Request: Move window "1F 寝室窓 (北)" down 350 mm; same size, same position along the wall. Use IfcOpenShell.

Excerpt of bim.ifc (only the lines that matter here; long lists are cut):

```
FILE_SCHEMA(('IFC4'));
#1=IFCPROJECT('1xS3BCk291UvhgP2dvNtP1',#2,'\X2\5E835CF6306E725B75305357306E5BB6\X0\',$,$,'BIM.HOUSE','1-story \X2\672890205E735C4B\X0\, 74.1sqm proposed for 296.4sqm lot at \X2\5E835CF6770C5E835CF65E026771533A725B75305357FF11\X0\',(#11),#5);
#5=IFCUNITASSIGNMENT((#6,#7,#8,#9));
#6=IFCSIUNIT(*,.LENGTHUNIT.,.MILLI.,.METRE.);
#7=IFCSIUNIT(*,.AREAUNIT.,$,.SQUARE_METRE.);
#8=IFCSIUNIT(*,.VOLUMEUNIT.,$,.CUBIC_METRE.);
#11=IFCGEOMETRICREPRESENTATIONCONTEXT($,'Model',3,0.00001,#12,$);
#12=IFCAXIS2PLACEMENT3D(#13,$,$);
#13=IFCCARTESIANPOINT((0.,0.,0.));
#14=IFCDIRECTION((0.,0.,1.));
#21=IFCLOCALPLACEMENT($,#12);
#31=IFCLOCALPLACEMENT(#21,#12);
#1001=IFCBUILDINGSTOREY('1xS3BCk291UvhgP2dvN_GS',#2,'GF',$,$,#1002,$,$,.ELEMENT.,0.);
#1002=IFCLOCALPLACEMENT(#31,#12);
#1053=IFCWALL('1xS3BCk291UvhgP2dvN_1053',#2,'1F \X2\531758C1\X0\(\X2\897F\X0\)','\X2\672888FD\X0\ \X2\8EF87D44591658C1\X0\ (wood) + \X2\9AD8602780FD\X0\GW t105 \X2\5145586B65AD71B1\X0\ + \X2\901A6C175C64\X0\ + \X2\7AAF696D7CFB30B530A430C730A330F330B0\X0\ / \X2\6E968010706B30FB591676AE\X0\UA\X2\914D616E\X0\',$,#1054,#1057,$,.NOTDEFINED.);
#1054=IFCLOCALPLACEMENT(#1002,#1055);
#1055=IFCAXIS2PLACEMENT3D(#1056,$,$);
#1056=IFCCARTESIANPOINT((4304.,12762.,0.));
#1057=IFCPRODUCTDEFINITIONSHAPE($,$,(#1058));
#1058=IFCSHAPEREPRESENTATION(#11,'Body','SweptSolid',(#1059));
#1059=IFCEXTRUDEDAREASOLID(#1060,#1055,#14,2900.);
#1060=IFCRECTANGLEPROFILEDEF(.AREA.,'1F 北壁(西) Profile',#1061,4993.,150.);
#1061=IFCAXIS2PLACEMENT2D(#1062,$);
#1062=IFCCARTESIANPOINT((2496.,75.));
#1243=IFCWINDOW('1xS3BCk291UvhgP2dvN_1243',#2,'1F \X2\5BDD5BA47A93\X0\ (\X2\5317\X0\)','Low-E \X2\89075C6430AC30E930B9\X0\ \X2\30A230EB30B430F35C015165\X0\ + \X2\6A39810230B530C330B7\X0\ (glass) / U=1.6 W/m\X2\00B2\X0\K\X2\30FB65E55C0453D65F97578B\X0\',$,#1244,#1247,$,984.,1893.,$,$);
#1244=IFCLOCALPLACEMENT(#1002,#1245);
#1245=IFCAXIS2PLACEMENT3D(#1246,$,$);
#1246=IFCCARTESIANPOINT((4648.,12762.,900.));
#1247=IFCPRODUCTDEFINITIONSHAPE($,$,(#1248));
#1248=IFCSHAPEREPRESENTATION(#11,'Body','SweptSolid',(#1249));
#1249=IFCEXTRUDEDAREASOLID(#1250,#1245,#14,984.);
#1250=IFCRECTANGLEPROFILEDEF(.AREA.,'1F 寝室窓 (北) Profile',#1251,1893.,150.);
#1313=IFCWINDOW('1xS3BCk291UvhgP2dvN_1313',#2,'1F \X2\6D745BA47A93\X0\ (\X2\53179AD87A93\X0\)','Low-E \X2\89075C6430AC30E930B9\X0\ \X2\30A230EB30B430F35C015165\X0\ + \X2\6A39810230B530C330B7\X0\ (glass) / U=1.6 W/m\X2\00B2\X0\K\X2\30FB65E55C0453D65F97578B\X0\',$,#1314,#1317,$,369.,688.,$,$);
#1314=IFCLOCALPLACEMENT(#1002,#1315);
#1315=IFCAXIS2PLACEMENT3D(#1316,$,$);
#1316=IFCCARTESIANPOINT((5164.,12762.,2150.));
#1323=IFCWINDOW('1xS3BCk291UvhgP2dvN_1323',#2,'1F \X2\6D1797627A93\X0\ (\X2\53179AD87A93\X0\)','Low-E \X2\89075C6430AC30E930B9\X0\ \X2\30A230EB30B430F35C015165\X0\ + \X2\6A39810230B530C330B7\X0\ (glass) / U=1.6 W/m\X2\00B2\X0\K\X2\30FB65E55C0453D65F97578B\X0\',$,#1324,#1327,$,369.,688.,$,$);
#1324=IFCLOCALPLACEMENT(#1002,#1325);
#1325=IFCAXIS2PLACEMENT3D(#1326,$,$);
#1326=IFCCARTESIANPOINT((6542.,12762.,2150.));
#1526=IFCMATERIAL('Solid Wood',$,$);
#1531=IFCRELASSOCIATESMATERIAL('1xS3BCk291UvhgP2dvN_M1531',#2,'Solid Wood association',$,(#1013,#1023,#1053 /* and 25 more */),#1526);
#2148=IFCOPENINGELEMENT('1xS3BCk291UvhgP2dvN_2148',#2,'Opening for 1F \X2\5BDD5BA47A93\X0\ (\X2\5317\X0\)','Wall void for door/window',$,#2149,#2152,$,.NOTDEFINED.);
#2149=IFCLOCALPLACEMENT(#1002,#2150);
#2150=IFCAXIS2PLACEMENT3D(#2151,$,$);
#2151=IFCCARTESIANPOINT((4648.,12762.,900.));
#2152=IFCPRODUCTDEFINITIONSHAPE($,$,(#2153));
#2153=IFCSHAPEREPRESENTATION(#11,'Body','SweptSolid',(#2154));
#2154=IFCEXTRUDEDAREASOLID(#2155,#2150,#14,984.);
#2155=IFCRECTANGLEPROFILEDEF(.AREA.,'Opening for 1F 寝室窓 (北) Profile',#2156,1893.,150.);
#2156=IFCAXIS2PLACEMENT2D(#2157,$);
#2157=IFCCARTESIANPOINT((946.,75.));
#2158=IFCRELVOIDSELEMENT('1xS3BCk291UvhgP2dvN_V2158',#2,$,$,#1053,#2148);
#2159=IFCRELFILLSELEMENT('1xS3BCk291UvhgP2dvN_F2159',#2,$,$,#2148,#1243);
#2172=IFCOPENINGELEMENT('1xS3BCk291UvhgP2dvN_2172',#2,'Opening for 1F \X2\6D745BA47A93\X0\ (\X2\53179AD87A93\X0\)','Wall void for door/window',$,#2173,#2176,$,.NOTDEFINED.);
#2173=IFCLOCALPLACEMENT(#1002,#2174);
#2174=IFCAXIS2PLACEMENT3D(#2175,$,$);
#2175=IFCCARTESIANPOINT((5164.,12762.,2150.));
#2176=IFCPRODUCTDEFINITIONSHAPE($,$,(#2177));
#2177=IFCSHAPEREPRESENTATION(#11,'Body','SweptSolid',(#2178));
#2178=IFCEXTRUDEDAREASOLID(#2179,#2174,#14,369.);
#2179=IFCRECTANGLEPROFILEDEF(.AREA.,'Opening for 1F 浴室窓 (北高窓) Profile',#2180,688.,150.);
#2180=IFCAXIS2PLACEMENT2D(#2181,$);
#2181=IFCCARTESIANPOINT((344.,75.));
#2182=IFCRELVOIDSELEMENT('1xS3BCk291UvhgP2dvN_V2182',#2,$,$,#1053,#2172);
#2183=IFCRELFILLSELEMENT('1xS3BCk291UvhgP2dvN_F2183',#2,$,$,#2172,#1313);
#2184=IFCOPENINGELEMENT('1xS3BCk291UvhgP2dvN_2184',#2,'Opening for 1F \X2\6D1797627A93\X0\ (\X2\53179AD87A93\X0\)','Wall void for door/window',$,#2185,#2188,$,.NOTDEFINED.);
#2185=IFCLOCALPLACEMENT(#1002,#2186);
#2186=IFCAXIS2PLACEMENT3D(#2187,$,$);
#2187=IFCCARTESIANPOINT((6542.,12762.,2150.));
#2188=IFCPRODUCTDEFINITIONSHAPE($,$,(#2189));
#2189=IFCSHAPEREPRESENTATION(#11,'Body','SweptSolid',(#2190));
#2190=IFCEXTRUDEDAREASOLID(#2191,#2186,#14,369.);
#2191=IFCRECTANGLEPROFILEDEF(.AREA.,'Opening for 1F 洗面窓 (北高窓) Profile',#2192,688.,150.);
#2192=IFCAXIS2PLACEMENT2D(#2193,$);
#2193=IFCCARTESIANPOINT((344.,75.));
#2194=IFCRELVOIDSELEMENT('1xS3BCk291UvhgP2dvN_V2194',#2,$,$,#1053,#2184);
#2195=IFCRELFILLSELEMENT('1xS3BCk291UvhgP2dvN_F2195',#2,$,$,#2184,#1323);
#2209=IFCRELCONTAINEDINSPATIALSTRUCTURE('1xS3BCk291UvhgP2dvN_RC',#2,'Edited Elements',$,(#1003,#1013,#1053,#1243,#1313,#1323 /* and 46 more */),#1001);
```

```python
import numpy as np
import ifcopenshell
import ifcopenshell.api.geometry
import ifcopenshell.util.placement
import ifcopenshell.util.unit

model = ifcopenshell.open("bim.ifc")
unit_scale = ifcopenshell.util.unit.calculate_unit_scale(model)

window = model.by_guid("1xS3BCk291UvhgP2dvN_1243")
opening = window.FillsVoids[0].RelatingOpeningElement
dz = -350.0

shift = np.array([0.0, 0.0, dz])
# The window is not placed relative to its opening, so move both.
for product in (opening, window):
    matrix = ifcopenshell.util.placement.get_local_placement(product.ObjectPlacement)
    matrix[:3, 3] += shift
    ifcopenshell.api.geometry.edit_object_placement(model, product=product, matrix=matrix, is_si=False)

print(f"moved by {dz * unit_scale:+.3f} m")

model.write("bim-out.ifc")
```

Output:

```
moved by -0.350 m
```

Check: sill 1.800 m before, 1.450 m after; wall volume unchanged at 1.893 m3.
